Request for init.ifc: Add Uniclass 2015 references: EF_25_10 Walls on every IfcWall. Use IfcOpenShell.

First a look at what the model holds.

```python
import ifcopenshell

model = ifcopenshell.open("init.ifc")
print(model.schema)
print("classifications:", [c.Name for c in model.by_type("IfcClassification")])
for ifc_class in ("IfcDoor", "IfcRoof", "IfcStair", "IfcWall", "IfcWindow"):
    print(ifc_class, len(model.by_type(ifc_class)))
```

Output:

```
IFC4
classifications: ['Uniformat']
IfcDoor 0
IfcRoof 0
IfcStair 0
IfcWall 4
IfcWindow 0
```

```python
import ifcopenshell
import ifcopenshell.api.classification

model = ifcopenshell.open("init.ifc")

system = ifcopenshell.api.classification.add_classification(model, classification="Uniclass 2015")

codes = {
    "IfcWall": ("EF_25_10", "Walls"),
}
for ifc_class, (code, name) in codes.items():
    products = model.by_type(ifc_class)
    ifcopenshell.api.classification.add_reference(
        model, products=products, classification=system, identification=code, name=name
    )
    print(code, len(products))

model.write("init_edited.ifc")
```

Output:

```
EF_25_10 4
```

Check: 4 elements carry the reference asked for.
